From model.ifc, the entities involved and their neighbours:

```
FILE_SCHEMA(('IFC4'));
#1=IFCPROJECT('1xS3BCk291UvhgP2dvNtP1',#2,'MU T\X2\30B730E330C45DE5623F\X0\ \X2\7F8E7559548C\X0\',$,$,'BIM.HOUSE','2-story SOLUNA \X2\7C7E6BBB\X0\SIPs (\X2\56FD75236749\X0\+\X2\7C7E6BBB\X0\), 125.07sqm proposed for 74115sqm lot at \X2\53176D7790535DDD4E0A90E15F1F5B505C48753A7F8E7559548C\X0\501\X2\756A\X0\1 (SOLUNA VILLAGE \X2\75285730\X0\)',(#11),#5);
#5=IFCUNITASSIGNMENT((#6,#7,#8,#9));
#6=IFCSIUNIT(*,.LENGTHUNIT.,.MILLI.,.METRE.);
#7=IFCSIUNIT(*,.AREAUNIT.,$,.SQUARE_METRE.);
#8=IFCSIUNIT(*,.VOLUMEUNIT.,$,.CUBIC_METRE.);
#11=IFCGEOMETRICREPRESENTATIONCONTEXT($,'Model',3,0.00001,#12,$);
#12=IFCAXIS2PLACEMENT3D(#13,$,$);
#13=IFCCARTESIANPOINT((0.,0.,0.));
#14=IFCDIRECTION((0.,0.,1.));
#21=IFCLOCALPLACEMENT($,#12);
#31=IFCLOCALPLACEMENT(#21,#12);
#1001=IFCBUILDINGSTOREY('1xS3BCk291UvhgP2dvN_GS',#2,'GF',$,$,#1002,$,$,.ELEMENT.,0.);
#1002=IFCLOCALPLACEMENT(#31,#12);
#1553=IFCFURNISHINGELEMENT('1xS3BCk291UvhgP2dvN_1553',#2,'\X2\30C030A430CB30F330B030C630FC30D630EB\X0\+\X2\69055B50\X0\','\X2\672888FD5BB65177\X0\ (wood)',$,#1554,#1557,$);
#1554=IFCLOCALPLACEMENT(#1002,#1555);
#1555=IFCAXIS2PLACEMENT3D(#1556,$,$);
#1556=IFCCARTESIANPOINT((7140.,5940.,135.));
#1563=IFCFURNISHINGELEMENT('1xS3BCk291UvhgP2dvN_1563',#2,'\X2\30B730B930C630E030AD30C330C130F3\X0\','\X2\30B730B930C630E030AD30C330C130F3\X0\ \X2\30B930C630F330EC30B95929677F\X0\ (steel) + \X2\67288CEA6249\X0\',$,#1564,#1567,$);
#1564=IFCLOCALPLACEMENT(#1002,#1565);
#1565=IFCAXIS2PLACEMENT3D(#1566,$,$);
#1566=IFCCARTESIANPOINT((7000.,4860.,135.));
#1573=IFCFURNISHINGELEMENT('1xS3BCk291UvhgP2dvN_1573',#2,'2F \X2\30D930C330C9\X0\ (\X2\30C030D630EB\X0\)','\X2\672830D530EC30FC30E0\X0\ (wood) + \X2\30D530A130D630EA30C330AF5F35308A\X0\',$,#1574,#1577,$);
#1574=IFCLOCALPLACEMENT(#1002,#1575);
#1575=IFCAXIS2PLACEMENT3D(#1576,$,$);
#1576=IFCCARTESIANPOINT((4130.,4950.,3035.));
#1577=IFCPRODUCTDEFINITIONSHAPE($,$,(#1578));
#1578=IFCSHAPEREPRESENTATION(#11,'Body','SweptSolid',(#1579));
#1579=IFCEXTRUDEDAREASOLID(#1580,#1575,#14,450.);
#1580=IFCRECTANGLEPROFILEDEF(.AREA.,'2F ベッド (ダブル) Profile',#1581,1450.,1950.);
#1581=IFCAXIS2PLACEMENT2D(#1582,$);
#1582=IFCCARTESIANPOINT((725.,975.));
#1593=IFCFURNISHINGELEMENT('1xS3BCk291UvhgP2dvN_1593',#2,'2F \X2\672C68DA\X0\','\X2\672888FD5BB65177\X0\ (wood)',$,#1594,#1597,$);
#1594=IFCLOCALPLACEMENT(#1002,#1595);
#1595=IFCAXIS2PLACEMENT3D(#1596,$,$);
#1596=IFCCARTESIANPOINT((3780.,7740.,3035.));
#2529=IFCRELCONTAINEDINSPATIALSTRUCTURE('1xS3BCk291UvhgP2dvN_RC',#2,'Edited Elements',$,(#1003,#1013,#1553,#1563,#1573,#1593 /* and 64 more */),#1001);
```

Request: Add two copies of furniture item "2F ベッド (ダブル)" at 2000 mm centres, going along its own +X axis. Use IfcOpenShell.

```python
import ifcopenshell
import ifcopenshell.api.geometry
import ifcopenshell.api.root
import ifcopenshell.util.element
import ifcopenshell.util.placement
import ifcopenshell.util.unit

model = ifcopenshell.open("model.ifc")
unit_scale = ifcopenshell.util.unit.calculate_unit_scale(model)


def reuse_history(source, copy):
    """copy_class also copies each property set's owner history, people and application; keep the originals."""
    for rel in copy.IsDefinedBy:
        if rel.is_a("IfcRelDefinesByProperties") and (history := rel.RelatingPropertyDefinition.OwnerHistory):
            rel.RelatingPropertyDefinition.OwnerHistory = source.OwnerHistory
            ifcopenshell.util.element.remove_deep2(model, history)


source = model.by_id(1573)
base = ifcopenshell.util.placement.get_local_placement(source.ObjectPlacement)
step = base[:3, 0] * 2 / unit_scale

for i in range(1, 3):
    copy = ifcopenshell.api.root.copy_class(model, product=source)
    copy.Representation = ifcopenshell.util.element.copy_deep(
        model, source.Representation, exclude=["IfcGeometricRepresentationContext", "IfcRepresentationMap"]
    )
    reuse_history(source, copy)
    matrix = base.copy()
    matrix[:3, 3] += i * step
    print("added at", matrix[:3, 3].round(3) + 0.0)
    ifcopenshell.api.geometry.edit_object_placement(model, product=copy, matrix=matrix, is_si=False)

model.write("model_edited.ifc")
```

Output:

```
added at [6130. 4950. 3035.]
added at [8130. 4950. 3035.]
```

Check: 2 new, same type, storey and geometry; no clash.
